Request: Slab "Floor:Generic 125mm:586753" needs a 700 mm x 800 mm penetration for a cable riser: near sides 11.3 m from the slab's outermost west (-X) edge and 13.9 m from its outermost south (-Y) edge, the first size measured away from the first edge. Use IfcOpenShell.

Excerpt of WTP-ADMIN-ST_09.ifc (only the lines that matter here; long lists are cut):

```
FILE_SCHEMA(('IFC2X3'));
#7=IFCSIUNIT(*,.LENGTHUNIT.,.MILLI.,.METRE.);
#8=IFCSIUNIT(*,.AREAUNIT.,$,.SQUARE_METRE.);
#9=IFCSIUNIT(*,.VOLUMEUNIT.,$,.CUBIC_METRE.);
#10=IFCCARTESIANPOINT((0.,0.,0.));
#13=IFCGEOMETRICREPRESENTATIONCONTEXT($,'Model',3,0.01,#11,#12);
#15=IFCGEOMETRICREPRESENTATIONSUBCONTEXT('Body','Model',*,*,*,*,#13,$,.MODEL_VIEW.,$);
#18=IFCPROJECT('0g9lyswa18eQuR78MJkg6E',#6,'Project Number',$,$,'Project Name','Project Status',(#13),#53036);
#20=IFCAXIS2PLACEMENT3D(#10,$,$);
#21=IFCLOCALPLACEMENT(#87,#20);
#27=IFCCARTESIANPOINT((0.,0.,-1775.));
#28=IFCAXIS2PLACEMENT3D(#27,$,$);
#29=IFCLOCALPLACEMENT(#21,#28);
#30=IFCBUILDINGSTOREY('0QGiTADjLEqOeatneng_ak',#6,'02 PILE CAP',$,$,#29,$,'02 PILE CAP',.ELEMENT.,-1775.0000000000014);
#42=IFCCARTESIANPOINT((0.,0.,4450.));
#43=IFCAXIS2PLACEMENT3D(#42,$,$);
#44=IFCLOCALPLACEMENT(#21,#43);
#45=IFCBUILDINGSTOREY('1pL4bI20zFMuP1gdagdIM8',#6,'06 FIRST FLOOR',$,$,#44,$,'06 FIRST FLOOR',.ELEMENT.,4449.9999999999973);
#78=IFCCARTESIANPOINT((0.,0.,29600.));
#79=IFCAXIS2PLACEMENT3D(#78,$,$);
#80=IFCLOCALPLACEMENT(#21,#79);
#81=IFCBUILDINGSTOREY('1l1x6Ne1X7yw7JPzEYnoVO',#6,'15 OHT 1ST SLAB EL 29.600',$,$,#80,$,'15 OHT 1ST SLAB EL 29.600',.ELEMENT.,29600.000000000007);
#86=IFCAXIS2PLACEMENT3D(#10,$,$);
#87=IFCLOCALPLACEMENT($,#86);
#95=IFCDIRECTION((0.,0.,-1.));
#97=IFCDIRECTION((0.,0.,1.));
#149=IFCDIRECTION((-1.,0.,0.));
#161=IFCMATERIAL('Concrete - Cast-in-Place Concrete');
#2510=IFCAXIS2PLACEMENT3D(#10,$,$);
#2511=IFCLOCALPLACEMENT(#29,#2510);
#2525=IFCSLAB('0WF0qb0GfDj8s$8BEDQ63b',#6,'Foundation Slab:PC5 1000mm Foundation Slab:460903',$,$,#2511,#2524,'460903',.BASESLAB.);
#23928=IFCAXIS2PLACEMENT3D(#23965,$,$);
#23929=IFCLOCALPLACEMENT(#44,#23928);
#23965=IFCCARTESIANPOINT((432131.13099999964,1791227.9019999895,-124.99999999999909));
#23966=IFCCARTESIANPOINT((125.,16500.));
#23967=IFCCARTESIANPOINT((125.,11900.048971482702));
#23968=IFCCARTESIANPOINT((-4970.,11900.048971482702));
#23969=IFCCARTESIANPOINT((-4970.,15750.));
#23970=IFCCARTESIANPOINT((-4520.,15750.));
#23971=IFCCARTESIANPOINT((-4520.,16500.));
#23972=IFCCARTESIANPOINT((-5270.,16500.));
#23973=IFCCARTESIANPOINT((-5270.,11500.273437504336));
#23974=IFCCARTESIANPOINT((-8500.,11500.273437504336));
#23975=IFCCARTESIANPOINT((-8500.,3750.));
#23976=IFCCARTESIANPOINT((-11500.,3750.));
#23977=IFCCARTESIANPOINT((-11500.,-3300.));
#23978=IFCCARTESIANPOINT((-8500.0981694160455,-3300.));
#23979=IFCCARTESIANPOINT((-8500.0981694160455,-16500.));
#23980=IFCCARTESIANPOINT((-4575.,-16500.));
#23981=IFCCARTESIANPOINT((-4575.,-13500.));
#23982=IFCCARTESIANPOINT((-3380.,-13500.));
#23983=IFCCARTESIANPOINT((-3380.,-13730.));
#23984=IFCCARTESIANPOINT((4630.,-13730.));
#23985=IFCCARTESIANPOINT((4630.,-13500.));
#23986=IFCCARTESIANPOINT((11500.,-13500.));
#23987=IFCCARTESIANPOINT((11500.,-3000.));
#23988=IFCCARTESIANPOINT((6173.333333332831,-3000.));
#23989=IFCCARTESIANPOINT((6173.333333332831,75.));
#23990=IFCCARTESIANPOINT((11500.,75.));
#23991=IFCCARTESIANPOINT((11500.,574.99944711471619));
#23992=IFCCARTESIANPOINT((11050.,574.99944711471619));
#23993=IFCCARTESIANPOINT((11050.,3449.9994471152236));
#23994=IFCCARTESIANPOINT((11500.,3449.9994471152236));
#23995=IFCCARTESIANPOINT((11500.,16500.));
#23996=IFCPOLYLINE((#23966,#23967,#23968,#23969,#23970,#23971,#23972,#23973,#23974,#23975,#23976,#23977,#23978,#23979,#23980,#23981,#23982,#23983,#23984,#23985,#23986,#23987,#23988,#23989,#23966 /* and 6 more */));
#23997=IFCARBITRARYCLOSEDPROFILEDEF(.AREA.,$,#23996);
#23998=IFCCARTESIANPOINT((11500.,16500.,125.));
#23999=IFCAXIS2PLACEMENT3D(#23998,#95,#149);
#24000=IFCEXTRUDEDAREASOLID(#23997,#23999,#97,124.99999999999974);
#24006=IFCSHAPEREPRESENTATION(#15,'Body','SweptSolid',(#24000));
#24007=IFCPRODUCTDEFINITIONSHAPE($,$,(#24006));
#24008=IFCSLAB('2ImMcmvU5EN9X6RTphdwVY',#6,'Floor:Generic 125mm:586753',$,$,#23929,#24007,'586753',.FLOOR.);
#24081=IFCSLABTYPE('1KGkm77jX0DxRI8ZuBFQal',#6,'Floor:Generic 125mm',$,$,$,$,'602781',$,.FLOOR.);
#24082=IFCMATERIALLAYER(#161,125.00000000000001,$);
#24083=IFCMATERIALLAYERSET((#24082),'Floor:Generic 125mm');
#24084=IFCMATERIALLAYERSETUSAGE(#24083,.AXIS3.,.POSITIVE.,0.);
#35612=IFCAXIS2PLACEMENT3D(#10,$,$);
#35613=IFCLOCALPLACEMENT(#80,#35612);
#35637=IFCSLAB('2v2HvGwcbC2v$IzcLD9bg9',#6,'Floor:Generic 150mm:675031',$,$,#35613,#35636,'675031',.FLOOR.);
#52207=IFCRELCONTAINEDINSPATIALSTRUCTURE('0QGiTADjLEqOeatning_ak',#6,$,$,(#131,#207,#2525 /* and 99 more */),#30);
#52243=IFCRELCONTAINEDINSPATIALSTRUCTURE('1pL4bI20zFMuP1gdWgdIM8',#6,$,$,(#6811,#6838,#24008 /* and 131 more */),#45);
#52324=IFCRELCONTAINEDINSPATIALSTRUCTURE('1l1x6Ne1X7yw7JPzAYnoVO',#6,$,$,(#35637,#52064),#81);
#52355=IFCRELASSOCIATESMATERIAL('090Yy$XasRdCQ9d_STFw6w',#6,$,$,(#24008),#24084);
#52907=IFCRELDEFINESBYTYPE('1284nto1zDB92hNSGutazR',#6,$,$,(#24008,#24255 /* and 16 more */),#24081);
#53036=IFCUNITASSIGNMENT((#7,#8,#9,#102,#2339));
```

```python
import numpy as np
import ifcopenshell
import ifcopenshell.api.feature
import ifcopenshell.api.geometry
import ifcopenshell.api.root
import ifcopenshell.geom
import ifcopenshell.util.placement
import ifcopenshell.util.representation
import ifcopenshell.util.shape
import ifcopenshell.util.unit

model = ifcopenshell.open("WTP-ADMIN-ST_09.ifc")
unit_scale = ifcopenshell.util.unit.calculate_unit_scale(model)
settings = ifcopenshell.geom.settings()


def volume(element):
    """Net volume in cubic metres, openings subtracted."""
    shape = ifcopenshell.geom.create_shape(settings, element)
    return ifcopenshell.util.shape.get_volume(shape.geometry)


slab = model.by_id(24008)
before = volume(slab)

# Extent in the slab's own axes, in metres. The edges named are its -X and -Y sides.
slab_shape = ifcopenshell.geom.create_shape(settings, slab)
vertices = ifcopenshell.util.shape.get_vertices(slab_shape.geometry)
x_min, y_min, bottom = vertices.min(axis=0)
top = vertices[:, 2].max()

opening = ifcopenshell.api.root.create_entity(model, ifc_class="IfcOpeningElement", name="Cable riser opening")
context = ifcopenshell.util.representation.get_context(model, "Model", "Body", "MODEL_VIEW")
width, depth = 0.7, 0.8
outline = [(0.0, 0.0), (width, 0.0), (width, depth), (0.0, depth), (0.0, 0.0)]
# Overshoot both faces by 50 mm so the cut is clean.
shape = ifcopenshell.api.geometry.add_slab_representation(
    model, context=context, depth=top - bottom + 0.1, polyline=outline
)
ifcopenshell.api.geometry.assign_representation(model, product=opening, representation=shape)

matrix = ifcopenshell.util.placement.get_local_placement(slab.ObjectPlacement)
matrix[:, 3] = matrix @ np.append(np.array([x_min + 11.3, y_min + 13.9, bottom - 0.05]) / unit_scale, 1.0)
ifcopenshell.api.geometry.edit_object_placement(model, product=opening, matrix=matrix, is_si=False)
ifcopenshell.api.feature.add_feature(model, feature=opening, element=slab)

after = volume(slab)

print(f"slab volume {before:.3f} -> {after:.3f} m3")

model.write("WTP-ADMIN-ST_09_v2.ifc")
```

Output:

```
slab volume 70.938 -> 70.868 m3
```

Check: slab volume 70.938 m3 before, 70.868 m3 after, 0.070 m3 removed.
